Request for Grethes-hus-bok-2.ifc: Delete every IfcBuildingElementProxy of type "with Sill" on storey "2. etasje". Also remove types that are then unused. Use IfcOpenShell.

First a look at what the model holds.

```python
import ifcopenshell
import ifcopenshell.util.element

model = ifcopenshell.open("Grethes-hus-bok-2.ifc")
print(model.schema)
storey = next(s for s in model.by_type("IfcBuildingStorey") if s.Name == "2. etasje")
proxies = [e for e in ifcopenshell.util.element.get_decomposition(storey) if e.is_a("IfcBuildingElementProxy")]
seen = {}
for e in proxies:
    element_type = ifcopenshell.util.element.get_type(e)
    name = element_type.Name if element_type not in (None, e) else None
    seen[name] = seen.get(name, 0) + 1
for name, count in sorted(seen.items(), key=str):
    print(count, "x", name)
```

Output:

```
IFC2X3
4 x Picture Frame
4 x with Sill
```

```python
import ifcopenshell
import ifcopenshell.api.root
import ifcopenshell.util.element

model = ifcopenshell.open("Grethes-hus-bok-2.ifc")

storey = next(s for s in model.by_type("IfcBuildingStorey") if s.Name == "2. etasje")
proxies = [e for e in ifcopenshell.util.element.get_decomposition(storey) if e.is_a("IfcBuildingElementProxy")]
targets = [e for e in proxies if (t := ifcopenshell.util.element.get_type(e)) not in (None, e) and t.Name == "with Sill"]
types = {ifcopenshell.util.element.get_type(e) for e in targets} - {None, *targets}

for e in targets:
    ifcopenshell.api.root.remove_product(model, product=e)
print(len(targets), "removed")

unused = [t for t in types if not ifcopenshell.util.element.get_types(t)]
for t in unused:
    ifcopenshell.api.root.remove_product(model, product=t)
print(len(unused), "unused types removed")

model.write("Grethes-hus-bok-2_v2.ifc")
```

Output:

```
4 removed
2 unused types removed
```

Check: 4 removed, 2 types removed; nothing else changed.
